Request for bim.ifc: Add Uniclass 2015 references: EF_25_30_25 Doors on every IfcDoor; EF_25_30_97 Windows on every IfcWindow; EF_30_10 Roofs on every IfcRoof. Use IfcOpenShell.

First a look at what the model holds.

```python
import ifcopenshell

model = ifcopenshell.open("bim.ifc")
print(model.schema)
print("classifications:", [c.Name for c in model.by_type("IfcClassification")])
for ifc_class in ("IfcDoor", "IfcRoof", "IfcStair", "IfcWall", "IfcWindow"):
    print(ifc_class, len(model.by_type(ifc_class)))
```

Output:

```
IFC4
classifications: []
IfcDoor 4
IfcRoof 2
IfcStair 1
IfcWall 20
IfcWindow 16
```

```python
import ifcopenshell
import ifcopenshell.api.classification

model = ifcopenshell.open("bim.ifc")

system = ifcopenshell.api.classification.add_classification(model, classification="Uniclass 2015")

codes = {
    "IfcDoor": ("EF_25_30_25", "Doors"),
    "IfcWindow": ("EF_25_30_97", "Windows"),
    "IfcRoof": ("EF_30_10", "Roofs"),
}
for ifc_class, (code, name) in codes.items():
    products = model.by_type(ifc_class)
    ifcopenshell.api.classification.add_reference(
        model, products=products, classification=system, identification=code, name=name
    )
    print(code, len(products))

model.write("bim_rev.ifc")
```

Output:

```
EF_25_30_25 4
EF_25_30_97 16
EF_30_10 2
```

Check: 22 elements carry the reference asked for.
